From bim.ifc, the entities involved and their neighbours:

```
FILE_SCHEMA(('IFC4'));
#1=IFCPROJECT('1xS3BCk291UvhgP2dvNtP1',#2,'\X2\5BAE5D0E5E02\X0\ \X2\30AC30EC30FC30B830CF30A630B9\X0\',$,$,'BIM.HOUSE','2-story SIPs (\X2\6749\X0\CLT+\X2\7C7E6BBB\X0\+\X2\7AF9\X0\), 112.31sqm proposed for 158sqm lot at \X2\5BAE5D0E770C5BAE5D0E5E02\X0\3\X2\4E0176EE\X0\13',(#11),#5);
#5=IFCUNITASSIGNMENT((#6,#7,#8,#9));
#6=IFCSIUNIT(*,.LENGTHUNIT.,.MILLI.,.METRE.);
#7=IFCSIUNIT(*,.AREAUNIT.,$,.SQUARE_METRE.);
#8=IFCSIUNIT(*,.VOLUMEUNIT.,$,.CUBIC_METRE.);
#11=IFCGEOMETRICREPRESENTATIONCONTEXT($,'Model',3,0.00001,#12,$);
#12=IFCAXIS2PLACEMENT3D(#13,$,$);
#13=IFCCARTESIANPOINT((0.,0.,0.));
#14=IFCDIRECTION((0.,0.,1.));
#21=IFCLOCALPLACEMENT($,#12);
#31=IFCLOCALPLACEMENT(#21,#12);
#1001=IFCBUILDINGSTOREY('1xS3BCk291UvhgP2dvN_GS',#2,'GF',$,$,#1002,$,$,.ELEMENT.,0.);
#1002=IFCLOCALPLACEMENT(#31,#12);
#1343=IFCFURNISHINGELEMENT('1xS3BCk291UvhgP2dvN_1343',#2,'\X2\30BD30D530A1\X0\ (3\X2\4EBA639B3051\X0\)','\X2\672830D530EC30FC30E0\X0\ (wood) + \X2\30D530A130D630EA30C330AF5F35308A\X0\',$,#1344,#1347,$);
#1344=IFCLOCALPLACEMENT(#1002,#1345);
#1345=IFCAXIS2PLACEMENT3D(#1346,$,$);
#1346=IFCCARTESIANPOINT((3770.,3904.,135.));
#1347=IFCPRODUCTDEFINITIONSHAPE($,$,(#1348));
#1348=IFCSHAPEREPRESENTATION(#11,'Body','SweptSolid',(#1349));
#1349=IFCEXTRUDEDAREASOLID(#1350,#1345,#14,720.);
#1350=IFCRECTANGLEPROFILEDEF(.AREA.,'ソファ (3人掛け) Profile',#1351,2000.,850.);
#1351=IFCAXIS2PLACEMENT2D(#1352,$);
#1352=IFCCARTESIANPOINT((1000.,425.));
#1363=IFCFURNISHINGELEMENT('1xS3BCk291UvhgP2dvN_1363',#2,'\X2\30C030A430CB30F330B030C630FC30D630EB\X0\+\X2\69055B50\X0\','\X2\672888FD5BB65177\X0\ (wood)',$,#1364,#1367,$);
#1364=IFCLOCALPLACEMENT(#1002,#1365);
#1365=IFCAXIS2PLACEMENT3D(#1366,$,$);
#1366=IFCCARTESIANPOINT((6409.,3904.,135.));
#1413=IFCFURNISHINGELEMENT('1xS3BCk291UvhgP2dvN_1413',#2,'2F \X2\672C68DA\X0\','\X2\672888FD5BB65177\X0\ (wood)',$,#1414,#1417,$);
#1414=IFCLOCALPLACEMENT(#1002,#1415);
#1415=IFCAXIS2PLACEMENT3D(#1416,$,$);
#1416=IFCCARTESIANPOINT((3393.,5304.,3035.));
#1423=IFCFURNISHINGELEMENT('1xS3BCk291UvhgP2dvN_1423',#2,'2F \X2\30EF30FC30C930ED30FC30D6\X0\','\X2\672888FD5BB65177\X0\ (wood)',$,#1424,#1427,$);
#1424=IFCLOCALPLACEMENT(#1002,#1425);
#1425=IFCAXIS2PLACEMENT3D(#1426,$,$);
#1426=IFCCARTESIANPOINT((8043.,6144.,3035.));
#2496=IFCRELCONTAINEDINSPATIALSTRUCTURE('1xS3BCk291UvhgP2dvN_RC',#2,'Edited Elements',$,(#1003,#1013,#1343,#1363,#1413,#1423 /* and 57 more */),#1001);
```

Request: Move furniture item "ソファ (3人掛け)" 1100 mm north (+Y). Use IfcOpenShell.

```python
import ifcopenshell
import ifcopenshell.api.geometry
import ifcopenshell.util.placement

model = ifcopenshell.open("bim.ifc")

item = model.by_guid("1xS3BCk291UvhgP2dvN_1343")
matrix = ifcopenshell.util.placement.get_local_placement(item.ObjectPlacement)
matrix[1, 3] += 1100.0
ifcopenshell.api.geometry.edit_object_placement(model, product=item, matrix=matrix, is_si=False)

print(ifcopenshell.util.placement.get_local_placement(item.ObjectPlacement).round(3) + 0.0)

model.write("bim-out.ifc")
```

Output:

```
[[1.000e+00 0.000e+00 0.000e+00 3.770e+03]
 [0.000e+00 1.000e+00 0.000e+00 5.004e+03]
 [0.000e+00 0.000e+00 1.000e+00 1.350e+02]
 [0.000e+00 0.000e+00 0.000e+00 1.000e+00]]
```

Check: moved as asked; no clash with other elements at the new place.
